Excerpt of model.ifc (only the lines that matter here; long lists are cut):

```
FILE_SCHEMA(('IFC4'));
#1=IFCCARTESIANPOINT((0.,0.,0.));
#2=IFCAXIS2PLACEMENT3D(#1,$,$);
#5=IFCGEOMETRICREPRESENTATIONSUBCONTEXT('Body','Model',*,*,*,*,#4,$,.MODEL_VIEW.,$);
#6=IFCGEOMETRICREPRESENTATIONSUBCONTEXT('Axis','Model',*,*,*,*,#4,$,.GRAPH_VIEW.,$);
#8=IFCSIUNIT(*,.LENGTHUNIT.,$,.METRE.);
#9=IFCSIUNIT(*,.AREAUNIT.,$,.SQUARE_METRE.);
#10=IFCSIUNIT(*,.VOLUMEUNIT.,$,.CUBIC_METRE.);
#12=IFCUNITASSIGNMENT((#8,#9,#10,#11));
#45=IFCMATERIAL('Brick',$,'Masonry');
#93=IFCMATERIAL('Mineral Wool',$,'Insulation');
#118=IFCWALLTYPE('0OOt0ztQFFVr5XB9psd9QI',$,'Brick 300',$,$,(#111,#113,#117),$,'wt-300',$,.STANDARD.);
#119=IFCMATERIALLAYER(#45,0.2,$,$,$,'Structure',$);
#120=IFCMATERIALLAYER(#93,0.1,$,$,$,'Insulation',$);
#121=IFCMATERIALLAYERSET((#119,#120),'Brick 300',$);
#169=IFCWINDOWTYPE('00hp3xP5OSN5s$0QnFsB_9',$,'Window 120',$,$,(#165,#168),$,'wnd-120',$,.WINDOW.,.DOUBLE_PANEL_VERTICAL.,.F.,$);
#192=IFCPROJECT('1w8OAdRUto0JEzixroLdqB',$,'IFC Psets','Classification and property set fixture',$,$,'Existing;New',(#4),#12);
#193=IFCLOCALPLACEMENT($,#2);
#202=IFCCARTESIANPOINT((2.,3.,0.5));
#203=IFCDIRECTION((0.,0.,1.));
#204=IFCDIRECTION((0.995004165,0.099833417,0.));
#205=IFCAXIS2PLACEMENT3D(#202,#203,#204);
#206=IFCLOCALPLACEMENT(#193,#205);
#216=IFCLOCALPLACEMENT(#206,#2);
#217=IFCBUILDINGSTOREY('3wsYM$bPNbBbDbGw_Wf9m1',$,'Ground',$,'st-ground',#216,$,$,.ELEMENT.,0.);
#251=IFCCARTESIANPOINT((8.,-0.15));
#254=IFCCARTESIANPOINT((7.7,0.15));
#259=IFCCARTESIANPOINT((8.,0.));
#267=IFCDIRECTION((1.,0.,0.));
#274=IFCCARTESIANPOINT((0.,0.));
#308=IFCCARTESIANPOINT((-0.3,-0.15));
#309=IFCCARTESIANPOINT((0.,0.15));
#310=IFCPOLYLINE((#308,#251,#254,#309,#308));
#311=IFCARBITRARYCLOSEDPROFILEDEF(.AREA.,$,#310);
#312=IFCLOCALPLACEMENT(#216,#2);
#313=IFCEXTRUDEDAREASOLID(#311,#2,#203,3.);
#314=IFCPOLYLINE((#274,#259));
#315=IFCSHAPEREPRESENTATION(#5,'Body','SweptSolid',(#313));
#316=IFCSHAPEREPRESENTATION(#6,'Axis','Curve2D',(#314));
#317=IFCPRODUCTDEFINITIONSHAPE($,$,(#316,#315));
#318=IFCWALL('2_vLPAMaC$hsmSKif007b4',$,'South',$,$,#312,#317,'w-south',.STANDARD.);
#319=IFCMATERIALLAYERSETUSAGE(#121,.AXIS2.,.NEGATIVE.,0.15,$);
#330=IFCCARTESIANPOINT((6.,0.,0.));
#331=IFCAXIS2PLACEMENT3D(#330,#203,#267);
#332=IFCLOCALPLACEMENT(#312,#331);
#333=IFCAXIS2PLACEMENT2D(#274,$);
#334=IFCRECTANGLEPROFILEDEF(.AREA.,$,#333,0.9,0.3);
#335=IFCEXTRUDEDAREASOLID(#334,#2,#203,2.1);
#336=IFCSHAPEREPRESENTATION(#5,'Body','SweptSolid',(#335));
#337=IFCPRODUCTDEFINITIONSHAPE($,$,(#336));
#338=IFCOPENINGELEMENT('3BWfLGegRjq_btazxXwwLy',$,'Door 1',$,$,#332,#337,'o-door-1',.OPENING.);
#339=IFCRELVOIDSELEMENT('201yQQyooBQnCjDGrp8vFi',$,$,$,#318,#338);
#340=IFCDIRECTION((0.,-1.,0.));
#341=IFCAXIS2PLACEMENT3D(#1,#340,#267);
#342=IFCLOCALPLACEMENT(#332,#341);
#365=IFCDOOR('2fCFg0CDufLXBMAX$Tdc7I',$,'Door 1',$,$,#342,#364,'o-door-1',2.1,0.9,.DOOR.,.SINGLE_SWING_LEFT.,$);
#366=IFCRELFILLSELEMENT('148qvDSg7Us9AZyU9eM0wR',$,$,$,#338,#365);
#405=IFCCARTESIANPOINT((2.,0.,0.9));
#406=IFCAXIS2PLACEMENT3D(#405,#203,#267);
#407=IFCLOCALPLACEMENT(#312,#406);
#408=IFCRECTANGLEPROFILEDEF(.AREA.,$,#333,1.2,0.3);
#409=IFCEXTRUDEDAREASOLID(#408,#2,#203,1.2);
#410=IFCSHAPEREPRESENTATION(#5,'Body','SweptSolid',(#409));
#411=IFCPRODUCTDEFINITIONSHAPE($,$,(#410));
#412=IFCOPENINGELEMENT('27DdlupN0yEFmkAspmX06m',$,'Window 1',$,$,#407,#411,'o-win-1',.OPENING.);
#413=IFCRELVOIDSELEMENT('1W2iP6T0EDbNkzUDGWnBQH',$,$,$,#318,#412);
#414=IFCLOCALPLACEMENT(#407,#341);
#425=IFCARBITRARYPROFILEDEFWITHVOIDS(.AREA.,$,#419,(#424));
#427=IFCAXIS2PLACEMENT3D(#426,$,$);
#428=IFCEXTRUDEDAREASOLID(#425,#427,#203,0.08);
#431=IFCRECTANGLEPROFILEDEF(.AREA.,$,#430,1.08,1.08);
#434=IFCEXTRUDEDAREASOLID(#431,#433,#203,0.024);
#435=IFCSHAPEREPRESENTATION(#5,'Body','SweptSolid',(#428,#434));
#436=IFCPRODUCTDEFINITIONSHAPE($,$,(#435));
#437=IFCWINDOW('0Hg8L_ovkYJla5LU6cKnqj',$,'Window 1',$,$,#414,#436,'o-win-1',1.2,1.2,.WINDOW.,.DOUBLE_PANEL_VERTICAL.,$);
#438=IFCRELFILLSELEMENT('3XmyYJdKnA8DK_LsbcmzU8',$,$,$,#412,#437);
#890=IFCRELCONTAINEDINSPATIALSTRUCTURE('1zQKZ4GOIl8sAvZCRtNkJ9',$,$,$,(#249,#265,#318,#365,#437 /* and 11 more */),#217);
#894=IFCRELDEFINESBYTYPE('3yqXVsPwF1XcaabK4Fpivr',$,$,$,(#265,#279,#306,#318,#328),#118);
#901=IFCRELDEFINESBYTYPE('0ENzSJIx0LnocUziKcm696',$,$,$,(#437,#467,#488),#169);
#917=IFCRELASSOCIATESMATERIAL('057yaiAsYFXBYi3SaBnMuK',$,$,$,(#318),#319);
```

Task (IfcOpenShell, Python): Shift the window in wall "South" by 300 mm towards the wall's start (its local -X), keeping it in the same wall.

```python
import ifcopenshell
import ifcopenshell.api.geometry
import ifcopenshell.util.placement

model = ifcopenshell.open("model.ifc")

window = model.by_guid("0Hg8L_ovkYJla5LU6cKnqj")
opening = window.FillsVoids[0].RelatingOpeningElement
wall = opening.VoidsElements[0].RelatingBuildingElement

wall_matrix = ifcopenshell.util.placement.get_local_placement(wall.ObjectPlacement)
shift = wall_matrix[:3, 0] * -0.3
before = ifcopenshell.util.placement.get_local_placement(window.ObjectPlacement)[:3, 3].copy()

# The window is placed relative to its opening, so it follows when the opening moves.
matrix = ifcopenshell.util.placement.get_local_placement(opening.ObjectPlacement)
matrix[:3, 3] += shift
ifcopenshell.api.geometry.edit_object_placement(
    model, product=opening, matrix=matrix, is_si=False, should_transform_children=True
)

after = ifcopenshell.util.placement.get_local_placement(window.ObjectPlacement)[:3, 3]
print("window moved by", (after - before).round(3) + 0.0)

model.write("model_edited.ifc")
```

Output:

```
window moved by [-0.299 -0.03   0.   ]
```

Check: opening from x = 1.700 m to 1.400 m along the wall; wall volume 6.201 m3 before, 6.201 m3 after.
